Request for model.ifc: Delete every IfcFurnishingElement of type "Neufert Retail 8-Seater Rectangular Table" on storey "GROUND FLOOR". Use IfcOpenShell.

First a look at what the model holds.

```python
import ifcopenshell
import ifcopenshell.util.element

model = ifcopenshell.open("model.ifc")
print(model.schema)
storey = next(s for s in model.by_type("IfcBuildingStorey") if s.Name == "GROUND FLOOR")
furniture = [e for e in ifcopenshell.util.element.get_decomposition(storey) if e.is_a("IfcFurnishingElement")]
seen = {}
for e in furniture:
    element_type = ifcopenshell.util.element.get_type(e)
    name = element_type.Name if element_type not in (None, e) else None
    seen[name] = seen.get(name, 0) + 1
for name, count in sorted(seen.items(), key=str):
    print(count, "x", name)
```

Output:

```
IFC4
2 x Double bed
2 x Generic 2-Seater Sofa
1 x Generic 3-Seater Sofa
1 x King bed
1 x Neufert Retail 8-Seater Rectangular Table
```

```python
import ifcopenshell
import ifcopenshell.api.root
import ifcopenshell.util.element

model = ifcopenshell.open("model.ifc")

storey = next(s for s in model.by_type("IfcBuildingStorey") if s.Name == "GROUND FLOOR")
furniture = [e for e in ifcopenshell.util.element.get_decomposition(storey) if e.is_a("IfcFurnishingElement")]
targets = [e for e in furniture if (t := ifcopenshell.util.element.get_type(e)) not in (None, e) and t.Name == "Neufert Retail 8-Seater Rectangular Table"]

for e in targets:
    ifcopenshell.api.root.remove_product(model, product=e)
print(len(targets), "removed")

model.write("model_updated.ifc")
```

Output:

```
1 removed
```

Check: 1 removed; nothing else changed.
